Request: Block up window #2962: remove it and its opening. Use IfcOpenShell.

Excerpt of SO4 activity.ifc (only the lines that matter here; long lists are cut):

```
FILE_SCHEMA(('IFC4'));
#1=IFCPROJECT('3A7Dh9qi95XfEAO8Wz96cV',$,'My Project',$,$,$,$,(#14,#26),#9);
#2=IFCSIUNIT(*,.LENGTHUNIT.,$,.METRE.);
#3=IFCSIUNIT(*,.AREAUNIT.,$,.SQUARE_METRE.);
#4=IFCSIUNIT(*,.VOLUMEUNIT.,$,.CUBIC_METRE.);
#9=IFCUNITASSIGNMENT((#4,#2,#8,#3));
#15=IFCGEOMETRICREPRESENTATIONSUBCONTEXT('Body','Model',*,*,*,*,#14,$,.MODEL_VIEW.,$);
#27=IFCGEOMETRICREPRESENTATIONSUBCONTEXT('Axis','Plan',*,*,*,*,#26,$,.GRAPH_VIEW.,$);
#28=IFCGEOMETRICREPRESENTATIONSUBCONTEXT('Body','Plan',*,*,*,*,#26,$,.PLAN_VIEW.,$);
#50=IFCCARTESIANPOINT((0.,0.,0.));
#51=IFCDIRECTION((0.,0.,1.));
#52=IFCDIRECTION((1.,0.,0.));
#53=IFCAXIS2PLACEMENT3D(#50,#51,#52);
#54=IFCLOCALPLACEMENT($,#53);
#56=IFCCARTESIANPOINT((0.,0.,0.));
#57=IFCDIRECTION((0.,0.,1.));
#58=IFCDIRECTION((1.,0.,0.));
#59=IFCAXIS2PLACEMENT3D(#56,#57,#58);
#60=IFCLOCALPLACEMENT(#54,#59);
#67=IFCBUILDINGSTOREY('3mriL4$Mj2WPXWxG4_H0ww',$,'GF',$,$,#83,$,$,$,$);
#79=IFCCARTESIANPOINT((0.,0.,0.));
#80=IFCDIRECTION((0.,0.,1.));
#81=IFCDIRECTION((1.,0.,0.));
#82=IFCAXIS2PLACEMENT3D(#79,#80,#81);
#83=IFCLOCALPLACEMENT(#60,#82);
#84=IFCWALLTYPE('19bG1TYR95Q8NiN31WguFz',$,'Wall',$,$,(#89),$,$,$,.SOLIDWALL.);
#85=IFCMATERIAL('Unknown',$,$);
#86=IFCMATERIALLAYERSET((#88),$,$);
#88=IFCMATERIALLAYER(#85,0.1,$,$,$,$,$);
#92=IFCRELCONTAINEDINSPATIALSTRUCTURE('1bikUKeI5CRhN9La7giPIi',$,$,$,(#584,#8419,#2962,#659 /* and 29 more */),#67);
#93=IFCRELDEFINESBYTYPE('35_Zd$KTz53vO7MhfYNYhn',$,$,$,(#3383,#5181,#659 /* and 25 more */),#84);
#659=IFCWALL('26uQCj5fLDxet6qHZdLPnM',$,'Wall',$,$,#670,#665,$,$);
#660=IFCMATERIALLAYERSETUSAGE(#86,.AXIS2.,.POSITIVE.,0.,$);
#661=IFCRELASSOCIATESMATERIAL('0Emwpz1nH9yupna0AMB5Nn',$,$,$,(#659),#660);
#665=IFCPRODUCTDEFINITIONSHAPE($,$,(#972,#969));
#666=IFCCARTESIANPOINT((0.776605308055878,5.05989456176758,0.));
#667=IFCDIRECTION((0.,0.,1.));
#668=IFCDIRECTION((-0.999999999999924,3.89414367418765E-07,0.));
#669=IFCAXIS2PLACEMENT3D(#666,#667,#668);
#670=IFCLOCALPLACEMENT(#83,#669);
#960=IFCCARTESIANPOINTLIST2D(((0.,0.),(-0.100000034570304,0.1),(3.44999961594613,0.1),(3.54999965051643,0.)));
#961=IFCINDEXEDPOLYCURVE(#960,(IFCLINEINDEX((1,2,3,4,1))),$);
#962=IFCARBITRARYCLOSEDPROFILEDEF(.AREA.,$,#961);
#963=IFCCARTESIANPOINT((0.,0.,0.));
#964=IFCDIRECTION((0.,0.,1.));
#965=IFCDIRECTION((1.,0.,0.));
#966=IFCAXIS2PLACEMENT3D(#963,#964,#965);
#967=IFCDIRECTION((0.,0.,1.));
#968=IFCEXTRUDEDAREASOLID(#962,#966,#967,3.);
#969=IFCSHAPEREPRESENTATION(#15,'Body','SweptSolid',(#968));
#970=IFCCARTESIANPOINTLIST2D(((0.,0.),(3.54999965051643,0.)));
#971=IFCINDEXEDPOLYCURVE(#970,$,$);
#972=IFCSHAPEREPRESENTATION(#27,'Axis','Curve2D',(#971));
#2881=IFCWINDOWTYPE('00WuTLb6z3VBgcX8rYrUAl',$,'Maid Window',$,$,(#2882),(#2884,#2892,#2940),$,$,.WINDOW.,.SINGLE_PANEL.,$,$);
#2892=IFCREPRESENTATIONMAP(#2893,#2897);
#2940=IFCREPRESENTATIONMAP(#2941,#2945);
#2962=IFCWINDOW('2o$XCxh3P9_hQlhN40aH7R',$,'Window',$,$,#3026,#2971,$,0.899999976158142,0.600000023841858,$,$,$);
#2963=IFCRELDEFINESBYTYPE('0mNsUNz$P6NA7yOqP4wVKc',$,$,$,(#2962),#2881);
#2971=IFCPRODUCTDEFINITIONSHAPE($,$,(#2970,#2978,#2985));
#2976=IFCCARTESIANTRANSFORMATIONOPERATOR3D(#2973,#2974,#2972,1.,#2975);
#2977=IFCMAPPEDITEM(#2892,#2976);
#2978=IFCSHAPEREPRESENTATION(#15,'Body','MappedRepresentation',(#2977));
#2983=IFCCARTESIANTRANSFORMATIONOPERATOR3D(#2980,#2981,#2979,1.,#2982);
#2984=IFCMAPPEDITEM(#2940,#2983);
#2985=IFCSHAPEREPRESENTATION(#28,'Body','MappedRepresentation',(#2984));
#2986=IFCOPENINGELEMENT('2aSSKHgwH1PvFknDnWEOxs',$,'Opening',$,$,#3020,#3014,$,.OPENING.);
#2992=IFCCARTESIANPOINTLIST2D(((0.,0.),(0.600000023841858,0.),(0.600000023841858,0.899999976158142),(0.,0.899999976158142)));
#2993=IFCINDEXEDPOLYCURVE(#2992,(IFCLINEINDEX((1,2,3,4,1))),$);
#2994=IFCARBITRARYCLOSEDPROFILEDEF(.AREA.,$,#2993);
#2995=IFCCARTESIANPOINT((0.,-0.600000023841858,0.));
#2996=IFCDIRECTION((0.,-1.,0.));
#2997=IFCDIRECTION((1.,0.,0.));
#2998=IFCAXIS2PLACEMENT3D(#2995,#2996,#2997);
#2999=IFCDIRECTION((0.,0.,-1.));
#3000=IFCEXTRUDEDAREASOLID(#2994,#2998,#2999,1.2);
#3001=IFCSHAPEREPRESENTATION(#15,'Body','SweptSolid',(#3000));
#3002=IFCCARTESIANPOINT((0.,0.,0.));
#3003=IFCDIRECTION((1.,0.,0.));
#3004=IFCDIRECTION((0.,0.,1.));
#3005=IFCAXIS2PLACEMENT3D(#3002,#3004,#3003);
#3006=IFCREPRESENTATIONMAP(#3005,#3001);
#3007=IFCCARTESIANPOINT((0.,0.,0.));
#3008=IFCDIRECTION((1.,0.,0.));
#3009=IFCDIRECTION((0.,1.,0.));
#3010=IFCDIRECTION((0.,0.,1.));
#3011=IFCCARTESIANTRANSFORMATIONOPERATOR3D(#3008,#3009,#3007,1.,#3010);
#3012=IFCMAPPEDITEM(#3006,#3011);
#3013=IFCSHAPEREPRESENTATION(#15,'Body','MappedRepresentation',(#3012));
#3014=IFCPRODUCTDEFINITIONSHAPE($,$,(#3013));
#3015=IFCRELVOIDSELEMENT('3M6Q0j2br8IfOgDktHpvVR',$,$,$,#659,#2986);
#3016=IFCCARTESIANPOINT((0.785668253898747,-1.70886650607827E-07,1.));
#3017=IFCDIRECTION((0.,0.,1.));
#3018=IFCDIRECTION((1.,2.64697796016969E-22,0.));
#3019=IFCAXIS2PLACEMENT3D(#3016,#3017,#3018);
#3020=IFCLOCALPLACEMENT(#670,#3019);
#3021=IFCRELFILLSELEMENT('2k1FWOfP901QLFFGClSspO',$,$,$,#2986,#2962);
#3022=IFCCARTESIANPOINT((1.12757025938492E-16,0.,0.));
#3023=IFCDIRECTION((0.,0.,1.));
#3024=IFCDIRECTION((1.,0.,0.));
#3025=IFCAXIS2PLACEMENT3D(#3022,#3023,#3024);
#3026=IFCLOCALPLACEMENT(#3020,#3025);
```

```python
import ifcopenshell
import ifcopenshell.api.feature
import ifcopenshell.api.root
import ifcopenshell.geom
import ifcopenshell.util.shape

model = ifcopenshell.open("SO4 activity.ifc")
settings = ifcopenshell.geom.settings()


def volume(element):
    """Net volume in cubic metres, openings subtracted."""
    shape = ifcopenshell.geom.create_shape(settings, element)
    return ifcopenshell.util.shape.get_volume(shape.geometry)


window = model.by_guid("2o$XCxh3P9_hQlhN40aH7R")
opening = window.FillsVoids[0].RelatingOpeningElement
wall = opening.VoidsElements[0].RelatingBuildingElement
before = volume(wall)

ifcopenshell.api.root.remove_product(model, product=window)
ifcopenshell.api.feature.remove_feature(model, feature=opening)

after = volume(wall)

print(f"wall volume {before:.3f} -> {after:.3f} m3")

model.write("SO4 activity_rev.ifc")
```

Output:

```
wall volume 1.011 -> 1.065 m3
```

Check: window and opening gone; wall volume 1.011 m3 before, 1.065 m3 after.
